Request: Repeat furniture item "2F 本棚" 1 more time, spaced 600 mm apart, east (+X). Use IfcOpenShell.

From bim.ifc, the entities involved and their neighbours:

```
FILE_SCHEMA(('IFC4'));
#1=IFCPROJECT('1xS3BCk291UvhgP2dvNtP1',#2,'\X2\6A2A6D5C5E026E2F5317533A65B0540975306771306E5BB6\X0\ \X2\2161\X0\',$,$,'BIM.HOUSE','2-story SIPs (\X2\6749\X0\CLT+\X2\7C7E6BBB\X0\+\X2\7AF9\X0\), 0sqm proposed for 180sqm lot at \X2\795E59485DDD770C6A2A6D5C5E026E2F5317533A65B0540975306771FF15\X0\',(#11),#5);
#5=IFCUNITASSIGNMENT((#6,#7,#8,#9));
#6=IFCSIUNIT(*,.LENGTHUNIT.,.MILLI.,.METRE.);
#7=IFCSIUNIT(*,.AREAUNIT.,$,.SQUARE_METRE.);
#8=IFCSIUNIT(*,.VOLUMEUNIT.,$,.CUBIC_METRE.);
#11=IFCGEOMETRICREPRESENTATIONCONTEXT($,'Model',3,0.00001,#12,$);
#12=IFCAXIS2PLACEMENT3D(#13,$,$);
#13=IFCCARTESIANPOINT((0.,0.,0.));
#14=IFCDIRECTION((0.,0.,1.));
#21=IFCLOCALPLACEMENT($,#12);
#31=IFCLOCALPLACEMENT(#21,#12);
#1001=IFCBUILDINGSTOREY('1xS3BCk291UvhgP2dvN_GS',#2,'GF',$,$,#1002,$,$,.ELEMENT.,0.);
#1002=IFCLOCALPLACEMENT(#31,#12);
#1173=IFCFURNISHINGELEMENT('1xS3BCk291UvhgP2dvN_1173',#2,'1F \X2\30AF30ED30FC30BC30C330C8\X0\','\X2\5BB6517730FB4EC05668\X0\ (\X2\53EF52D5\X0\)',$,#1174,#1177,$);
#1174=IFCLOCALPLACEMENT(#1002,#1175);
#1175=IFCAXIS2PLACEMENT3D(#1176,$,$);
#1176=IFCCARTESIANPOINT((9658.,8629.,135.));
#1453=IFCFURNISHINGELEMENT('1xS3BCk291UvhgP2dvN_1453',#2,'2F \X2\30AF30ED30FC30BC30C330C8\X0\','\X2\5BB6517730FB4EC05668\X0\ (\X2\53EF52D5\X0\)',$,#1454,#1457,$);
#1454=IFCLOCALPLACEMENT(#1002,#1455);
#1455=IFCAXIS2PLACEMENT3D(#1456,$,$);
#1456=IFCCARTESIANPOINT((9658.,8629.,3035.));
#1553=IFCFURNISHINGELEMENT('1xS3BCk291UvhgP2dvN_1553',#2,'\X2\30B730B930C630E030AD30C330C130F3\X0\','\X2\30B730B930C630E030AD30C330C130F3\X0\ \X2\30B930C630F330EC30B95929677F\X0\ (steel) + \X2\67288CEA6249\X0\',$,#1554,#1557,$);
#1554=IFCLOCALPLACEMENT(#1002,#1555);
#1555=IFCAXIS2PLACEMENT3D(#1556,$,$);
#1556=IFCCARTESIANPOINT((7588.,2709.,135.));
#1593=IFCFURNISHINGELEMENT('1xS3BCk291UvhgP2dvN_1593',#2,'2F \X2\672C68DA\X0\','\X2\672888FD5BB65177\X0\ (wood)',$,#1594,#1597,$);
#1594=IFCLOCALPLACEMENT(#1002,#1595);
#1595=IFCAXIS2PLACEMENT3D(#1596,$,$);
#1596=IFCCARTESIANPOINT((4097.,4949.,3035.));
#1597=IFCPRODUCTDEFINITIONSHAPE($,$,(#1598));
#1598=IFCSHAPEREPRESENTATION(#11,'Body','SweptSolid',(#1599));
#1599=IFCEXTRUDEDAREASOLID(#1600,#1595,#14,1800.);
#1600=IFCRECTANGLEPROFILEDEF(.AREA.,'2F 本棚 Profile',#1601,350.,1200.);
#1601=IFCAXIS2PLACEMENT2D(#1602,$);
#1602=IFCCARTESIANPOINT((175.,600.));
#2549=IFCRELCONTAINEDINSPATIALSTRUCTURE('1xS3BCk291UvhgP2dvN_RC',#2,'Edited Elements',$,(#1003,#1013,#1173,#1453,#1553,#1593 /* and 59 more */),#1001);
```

```python
import numpy as np
import ifcopenshell
import ifcopenshell.api.geometry
import ifcopenshell.api.root
import ifcopenshell.util.element
import ifcopenshell.util.placement
import ifcopenshell.util.unit

model = ifcopenshell.open("bim.ifc")
unit_scale = ifcopenshell.util.unit.calculate_unit_scale(model)


def reuse_history(source, copy):
    """copy_class also copies each property set's owner history, people and application; keep the originals."""
    for rel in copy.IsDefinedBy:
        if rel.is_a("IfcRelDefinesByProperties") and (history := rel.RelatingPropertyDefinition.OwnerHistory):
            rel.RelatingPropertyDefinition.OwnerHistory = source.OwnerHistory
            ifcopenshell.util.element.remove_deep2(model, history)


source = model.by_id(1593)
base = ifcopenshell.util.placement.get_local_placement(source.ObjectPlacement)
step = np.array([1.0, 0.0, 0.0]) * 0.6 / unit_scale

for i in range(1, 2):
    copy = ifcopenshell.api.root.copy_class(model, product=source)
    copy.Representation = ifcopenshell.util.element.copy_deep(
        model, source.Representation, exclude=["IfcGeometricRepresentationContext", "IfcRepresentationMap"]
    )
    reuse_history(source, copy)
    matrix = base.copy()
    matrix[:3, 3] += i * step
    print("added at", matrix[:3, 3].round(3) + 0.0)
    ifcopenshell.api.geometry.edit_object_placement(model, product=copy, matrix=matrix, is_si=False)

model.write("bim_v2.ifc")
```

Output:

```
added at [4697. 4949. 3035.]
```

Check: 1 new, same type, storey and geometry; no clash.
